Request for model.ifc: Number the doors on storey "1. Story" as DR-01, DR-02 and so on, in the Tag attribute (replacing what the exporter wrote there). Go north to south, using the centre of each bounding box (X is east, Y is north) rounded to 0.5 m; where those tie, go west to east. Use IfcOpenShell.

First a look at what the model holds.

```python
import ifcopenshell
import ifcopenshell.util.element
import ifcopenshell.util.placement

model = ifcopenshell.open("model.ifc")
print(model.schema)
storey = next(s for s in model.by_type("IfcBuildingStorey") if s.Name == "1. Story")
doors = [e for e in ifcopenshell.util.element.get_decomposition(storey) if e.is_a("IfcDoor")]
for e in sorted(doors, key=lambda e: e.id()):
    origin = ifcopenshell.util.placement.get_local_placement(e.ObjectPlacement)[:3, 3]
    print(e.id(), e.Tag, e.Name, origin.round(2) + 0.0, sep=" | ")
```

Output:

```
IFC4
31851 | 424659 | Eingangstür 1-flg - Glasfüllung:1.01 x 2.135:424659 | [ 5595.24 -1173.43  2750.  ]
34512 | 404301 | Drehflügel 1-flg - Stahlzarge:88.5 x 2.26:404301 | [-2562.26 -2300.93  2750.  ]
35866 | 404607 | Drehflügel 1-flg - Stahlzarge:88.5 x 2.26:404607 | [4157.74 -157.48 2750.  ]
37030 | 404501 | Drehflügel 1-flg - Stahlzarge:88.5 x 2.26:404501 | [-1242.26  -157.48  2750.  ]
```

```python
import ifcopenshell
import ifcopenshell.geom
import ifcopenshell.util.element
import ifcopenshell.util.shape

model = ifcopenshell.open("model.ifc")
settings = ifcopenshell.geom.settings()
settings.set("use-world-coords", True)


def centre(element):
    shape = ifcopenshell.geom.create_shape(settings, element)
    return ifcopenshell.util.shape.get_bbox_centroid(shape.geometry)


storey = next(s for s in model.by_type("IfcBuildingStorey") if s.Name == "1. Story")
doors = [e for e in ifcopenshell.util.element.get_decomposition(storey) if e.is_a("IfcDoor")]

# Insertion points can sit at a corner or the storey origin, so sort by the geometry (in metres).
centres = {e: centre(e) for e in doors}
doors.sort(key=lambda e: (-round(centres[e][1] / 0.5), centres[e][0]))

for i, e in enumerate(doors, start=1):
    number = f"DR-{i:02d}"
    e.Tag = number
    print(e.id(), number)

model.write("model_v2.ifc")
```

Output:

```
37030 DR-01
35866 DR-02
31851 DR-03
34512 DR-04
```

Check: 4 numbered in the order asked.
